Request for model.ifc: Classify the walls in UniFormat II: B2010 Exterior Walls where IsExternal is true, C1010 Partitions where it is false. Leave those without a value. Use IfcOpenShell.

First a look at what the model holds.

```python
import ifcopenshell
import ifcopenshell.util.element

model = ifcopenshell.open("model.ifc")
print(model.schema)
print("classifications:", [c.Name for c in model.by_type("IfcClassification")])
values = [ifcopenshell.util.element.get_pset(e, "Pset_WallCommon", "IsExternal") for e in model.by_type("IfcWall")]
for value in (True, False, None):
    print("IsExternal", value, values.count(value))
```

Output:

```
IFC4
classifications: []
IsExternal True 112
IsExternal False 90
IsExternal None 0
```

```python
import ifcopenshell
import ifcopenshell.api.classification
import ifcopenshell.util.element

model = ifcopenshell.open("model.ifc")

system = ifcopenshell.api.classification.add_classification(model, classification="UniFormat II")

walls = model.by_type("IfcWall")
external = {e: ifcopenshell.util.element.get_pset(e, "Pset_WallCommon", "IsExternal") for e in walls}
for flag, code, name in ((True, "B2010", "Exterior Walls"), (False, "C1010", "Partitions")):
    products = [e for e in walls if external[e] is flag]
    ifcopenshell.api.classification.add_reference(
        model, products=products, classification=system, identification=code, name=name
    )
    print(code, len(products))

model.write("model_v2.ifc")
```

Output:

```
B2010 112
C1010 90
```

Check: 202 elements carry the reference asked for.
